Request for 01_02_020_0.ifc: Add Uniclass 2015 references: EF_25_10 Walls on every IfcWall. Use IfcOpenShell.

First a look at what the model holds.

```python
import ifcopenshell

model = ifcopenshell.open("01_02_020_0.ifc")
print(model.schema)
print("classifications:", [c.Name for c in model.by_type("IfcClassification")])
for ifc_class in ("IfcDoor", "IfcRoof", "IfcStair", "IfcWall", "IfcWindow"):
    print(ifc_class, len(model.by_type(ifc_class)))
```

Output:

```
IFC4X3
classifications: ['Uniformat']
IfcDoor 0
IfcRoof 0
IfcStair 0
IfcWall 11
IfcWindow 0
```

```python
import ifcopenshell
import ifcopenshell.api.classification

model = ifcopenshell.open("01_02_020_0.ifc")

system = ifcopenshell.api.classification.add_classification(model, classification="Uniclass 2015")

codes = {
    "IfcWall": ("EF_25_10", "Walls"),
}
for ifc_class, (code, name) in codes.items():
    products = model.by_type(ifc_class)
    ifcopenshell.api.classification.add_reference(
        model, products=products, classification=system, identification=code, name=name
    )
    print(code, len(products))

model.write("01_02_020_0-out.ifc")
```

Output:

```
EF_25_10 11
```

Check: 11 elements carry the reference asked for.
